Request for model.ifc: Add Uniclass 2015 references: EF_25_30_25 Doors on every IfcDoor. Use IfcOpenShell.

First a look at what the model holds.

```python
import ifcopenshell

model = ifcopenshell.open("model.ifc")
print(model.schema)
print("classifications:", [c.Name for c in model.by_type("IfcClassification")])
for ifc_class in ("IfcDoor", "IfcRoof", "IfcStair", "IfcWall", "IfcWindow"):
    print(ifc_class, len(model.by_type(ifc_class)))
```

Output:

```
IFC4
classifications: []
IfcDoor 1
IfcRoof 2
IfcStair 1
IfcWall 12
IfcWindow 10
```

```python
import ifcopenshell
import ifcopenshell.api.classification

model = ifcopenshell.open("model.ifc")

system = ifcopenshell.api.classification.add_classification(model, classification="Uniclass 2015")

codes = {
    "IfcDoor": ("EF_25_30_25", "Doors"),
}
for ifc_class, (code, name) in codes.items():
    products = model.by_type(ifc_class)
    ifcopenshell.api.classification.add_reference(
        model, products=products, classification=system, identification=code, name=name
    )
    print(code, len(products))

model.write("model_v2.ifc")
```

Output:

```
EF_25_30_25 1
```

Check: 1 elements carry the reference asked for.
